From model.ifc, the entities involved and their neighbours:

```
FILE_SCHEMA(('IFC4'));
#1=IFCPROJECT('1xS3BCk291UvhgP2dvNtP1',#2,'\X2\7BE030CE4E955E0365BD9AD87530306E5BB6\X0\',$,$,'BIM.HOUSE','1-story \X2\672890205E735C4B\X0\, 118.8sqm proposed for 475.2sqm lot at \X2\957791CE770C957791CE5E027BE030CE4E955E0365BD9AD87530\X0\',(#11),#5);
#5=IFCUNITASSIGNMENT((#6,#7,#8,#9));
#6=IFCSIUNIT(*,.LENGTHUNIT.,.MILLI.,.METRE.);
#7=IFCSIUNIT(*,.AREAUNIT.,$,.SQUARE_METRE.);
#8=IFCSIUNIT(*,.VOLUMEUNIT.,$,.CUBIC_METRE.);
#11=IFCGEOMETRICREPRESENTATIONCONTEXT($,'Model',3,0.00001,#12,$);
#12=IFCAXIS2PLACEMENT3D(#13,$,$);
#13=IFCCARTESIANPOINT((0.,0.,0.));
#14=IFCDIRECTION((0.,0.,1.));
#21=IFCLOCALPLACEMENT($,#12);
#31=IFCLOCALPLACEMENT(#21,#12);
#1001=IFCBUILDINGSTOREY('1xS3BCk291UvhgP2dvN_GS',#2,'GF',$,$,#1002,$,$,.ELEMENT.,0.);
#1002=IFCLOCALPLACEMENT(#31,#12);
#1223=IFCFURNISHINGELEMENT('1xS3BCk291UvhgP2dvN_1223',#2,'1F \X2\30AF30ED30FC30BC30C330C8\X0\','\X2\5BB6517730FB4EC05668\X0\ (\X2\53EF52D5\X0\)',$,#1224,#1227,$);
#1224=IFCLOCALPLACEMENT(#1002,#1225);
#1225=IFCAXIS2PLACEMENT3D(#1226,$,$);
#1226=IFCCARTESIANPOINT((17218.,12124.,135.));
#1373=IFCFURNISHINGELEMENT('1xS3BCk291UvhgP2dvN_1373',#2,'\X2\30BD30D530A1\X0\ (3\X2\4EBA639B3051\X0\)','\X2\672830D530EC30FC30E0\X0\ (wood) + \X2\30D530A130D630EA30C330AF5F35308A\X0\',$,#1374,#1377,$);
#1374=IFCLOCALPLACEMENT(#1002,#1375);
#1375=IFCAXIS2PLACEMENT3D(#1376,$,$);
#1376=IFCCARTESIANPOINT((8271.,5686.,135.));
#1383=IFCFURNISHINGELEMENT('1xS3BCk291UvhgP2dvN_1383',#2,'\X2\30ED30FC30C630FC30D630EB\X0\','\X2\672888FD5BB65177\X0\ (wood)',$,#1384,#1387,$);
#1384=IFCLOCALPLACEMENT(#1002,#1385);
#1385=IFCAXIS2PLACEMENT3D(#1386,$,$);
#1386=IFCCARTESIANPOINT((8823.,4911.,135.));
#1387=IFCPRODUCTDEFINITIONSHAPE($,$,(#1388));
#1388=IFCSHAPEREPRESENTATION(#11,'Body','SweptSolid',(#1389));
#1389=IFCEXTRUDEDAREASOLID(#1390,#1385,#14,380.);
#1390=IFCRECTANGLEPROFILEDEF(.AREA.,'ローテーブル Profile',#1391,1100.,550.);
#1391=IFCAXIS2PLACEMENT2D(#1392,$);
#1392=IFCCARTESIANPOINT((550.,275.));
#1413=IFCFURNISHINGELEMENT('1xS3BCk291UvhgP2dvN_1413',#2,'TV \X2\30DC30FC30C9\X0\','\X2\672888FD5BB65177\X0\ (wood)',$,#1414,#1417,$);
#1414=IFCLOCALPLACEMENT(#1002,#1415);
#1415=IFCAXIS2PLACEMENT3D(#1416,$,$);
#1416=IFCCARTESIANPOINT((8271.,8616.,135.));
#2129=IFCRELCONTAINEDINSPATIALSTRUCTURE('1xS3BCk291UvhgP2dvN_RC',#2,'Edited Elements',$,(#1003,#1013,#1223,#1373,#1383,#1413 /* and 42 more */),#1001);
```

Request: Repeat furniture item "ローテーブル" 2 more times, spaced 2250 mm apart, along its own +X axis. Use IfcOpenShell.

```python
import ifcopenshell
import ifcopenshell.api.geometry
import ifcopenshell.api.root
import ifcopenshell.util.element
import ifcopenshell.util.placement

model = ifcopenshell.open("model.ifc")


def reuse_history(source, copy):
    """copy_class also copies each property set's owner history, people and application; keep the originals."""
    for rel in copy.IsDefinedBy:
        if rel.is_a("IfcRelDefinesByProperties") and (history := rel.RelatingPropertyDefinition.OwnerHistory):
            rel.RelatingPropertyDefinition.OwnerHistory = source.OwnerHistory
            ifcopenshell.util.element.remove_deep2(model, history)


source = model.by_guid("1xS3BCk291UvhgP2dvN_1383")
base = ifcopenshell.util.placement.get_local_placement(source.ObjectPlacement)
step = base[:3, 0] * 2250.0

for i in range(1, 3):
    copy = ifcopenshell.api.root.copy_class(model, product=source)
    copy.Representation = ifcopenshell.util.element.copy_deep(
        model, source.Representation, exclude=["IfcGeometricRepresentationContext", "IfcRepresentationMap"]
    )
    reuse_history(source, copy)
    matrix = base.copy()
    matrix[:3, 3] += i * step
    print("added at", matrix[:3, 3].round(3) + 0.0)
    ifcopenshell.api.geometry.edit_object_placement(model, product=copy, matrix=matrix, is_si=False)

model.write("model_v2.ifc")
```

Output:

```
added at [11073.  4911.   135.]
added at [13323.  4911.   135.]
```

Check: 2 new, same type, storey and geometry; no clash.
